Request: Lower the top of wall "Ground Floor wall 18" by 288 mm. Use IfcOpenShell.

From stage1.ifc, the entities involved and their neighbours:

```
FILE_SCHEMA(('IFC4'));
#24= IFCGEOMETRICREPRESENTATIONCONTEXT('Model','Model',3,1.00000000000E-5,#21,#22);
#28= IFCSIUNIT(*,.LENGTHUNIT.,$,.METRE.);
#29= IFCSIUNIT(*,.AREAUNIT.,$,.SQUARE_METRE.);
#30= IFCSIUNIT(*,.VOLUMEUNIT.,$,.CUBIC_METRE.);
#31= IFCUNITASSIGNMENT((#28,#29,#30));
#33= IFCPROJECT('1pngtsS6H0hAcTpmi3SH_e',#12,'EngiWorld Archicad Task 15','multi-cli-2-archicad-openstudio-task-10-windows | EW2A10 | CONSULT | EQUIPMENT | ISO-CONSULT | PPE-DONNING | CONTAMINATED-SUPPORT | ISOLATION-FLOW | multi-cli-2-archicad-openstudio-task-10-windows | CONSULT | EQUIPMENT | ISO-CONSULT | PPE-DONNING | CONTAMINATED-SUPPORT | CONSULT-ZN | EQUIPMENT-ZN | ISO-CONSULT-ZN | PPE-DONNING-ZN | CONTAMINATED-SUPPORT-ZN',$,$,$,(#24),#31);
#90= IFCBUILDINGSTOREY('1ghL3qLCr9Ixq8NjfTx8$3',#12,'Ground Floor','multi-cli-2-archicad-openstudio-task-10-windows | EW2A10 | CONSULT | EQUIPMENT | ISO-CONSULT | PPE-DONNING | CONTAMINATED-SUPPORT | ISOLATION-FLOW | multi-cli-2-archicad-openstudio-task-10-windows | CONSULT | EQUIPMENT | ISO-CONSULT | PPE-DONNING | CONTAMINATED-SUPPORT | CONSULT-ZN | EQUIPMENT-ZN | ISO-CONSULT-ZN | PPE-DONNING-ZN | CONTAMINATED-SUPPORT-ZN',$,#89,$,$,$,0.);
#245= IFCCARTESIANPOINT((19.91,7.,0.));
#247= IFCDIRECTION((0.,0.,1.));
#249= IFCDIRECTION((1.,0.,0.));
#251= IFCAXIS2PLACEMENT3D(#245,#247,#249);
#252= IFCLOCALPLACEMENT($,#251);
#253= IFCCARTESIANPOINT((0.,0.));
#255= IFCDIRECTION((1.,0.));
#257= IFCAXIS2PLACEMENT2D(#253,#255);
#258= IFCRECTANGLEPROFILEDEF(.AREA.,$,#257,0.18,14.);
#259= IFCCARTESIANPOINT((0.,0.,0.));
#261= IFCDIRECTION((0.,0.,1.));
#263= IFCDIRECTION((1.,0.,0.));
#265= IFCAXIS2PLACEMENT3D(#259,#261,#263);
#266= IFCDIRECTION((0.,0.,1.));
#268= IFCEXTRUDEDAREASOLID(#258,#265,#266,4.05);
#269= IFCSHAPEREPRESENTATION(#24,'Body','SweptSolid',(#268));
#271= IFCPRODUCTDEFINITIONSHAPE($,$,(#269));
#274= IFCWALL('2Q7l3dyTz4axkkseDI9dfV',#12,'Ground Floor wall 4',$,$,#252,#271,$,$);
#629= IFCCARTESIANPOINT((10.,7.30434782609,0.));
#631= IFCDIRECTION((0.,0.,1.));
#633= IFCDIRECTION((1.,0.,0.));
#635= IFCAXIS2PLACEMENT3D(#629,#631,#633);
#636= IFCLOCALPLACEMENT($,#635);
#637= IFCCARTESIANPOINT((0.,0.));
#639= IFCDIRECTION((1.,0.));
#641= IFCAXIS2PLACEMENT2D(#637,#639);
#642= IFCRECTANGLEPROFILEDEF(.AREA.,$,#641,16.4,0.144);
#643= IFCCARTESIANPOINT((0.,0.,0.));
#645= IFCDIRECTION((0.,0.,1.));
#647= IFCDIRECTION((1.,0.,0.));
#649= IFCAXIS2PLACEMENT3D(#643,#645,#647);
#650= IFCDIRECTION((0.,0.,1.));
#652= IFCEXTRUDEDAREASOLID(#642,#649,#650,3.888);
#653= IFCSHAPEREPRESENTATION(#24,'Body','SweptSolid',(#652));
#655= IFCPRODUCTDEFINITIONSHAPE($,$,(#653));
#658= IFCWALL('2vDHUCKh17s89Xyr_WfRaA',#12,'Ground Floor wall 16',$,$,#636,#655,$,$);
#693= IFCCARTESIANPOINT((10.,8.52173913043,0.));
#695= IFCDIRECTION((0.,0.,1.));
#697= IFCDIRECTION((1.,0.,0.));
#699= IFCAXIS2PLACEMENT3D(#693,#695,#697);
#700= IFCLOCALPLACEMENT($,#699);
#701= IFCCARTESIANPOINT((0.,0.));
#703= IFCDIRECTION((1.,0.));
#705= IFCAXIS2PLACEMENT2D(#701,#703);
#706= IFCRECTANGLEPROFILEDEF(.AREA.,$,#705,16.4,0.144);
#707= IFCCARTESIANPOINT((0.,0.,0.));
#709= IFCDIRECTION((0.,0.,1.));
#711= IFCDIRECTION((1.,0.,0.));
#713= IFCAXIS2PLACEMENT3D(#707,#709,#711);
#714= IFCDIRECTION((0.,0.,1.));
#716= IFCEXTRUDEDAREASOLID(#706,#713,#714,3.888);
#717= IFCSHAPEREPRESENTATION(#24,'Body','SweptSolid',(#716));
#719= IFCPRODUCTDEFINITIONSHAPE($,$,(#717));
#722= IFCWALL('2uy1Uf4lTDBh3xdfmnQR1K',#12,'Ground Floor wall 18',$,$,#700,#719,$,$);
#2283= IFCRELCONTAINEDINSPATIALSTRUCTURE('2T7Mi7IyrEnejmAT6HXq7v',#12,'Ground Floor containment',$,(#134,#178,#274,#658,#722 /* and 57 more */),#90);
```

```python
import ifcopenshell
import ifcopenshell.geom
import ifcopenshell.util.shape

model = ifcopenshell.open("stage1.ifc")
settings = ifcopenshell.geom.settings()


def volume(element):
    """Net volume in cubic metres, openings subtracted."""
    shape = ifcopenshell.geom.create_shape(settings, element)
    return ifcopenshell.util.shape.get_volume(shape.geometry)


wall = model.by_guid("2uy1Uf4lTDBh3xdfmnQR1K")
before = volume(wall)

body = next(r for r in wall.Representation.Representations if r.RepresentationIdentifier == "Body")
solid = body.Items[0]
old_height = solid.Depth
solid.Depth -= 0.288
after = volume(wall)

print(f"height {old_height:g} -> {solid.Depth:g}, volume {before:.3f} -> {after:.3f} m3")

model.write("stage1_edited.ifc")
```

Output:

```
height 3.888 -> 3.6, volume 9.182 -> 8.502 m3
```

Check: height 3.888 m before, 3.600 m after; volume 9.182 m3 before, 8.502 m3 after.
